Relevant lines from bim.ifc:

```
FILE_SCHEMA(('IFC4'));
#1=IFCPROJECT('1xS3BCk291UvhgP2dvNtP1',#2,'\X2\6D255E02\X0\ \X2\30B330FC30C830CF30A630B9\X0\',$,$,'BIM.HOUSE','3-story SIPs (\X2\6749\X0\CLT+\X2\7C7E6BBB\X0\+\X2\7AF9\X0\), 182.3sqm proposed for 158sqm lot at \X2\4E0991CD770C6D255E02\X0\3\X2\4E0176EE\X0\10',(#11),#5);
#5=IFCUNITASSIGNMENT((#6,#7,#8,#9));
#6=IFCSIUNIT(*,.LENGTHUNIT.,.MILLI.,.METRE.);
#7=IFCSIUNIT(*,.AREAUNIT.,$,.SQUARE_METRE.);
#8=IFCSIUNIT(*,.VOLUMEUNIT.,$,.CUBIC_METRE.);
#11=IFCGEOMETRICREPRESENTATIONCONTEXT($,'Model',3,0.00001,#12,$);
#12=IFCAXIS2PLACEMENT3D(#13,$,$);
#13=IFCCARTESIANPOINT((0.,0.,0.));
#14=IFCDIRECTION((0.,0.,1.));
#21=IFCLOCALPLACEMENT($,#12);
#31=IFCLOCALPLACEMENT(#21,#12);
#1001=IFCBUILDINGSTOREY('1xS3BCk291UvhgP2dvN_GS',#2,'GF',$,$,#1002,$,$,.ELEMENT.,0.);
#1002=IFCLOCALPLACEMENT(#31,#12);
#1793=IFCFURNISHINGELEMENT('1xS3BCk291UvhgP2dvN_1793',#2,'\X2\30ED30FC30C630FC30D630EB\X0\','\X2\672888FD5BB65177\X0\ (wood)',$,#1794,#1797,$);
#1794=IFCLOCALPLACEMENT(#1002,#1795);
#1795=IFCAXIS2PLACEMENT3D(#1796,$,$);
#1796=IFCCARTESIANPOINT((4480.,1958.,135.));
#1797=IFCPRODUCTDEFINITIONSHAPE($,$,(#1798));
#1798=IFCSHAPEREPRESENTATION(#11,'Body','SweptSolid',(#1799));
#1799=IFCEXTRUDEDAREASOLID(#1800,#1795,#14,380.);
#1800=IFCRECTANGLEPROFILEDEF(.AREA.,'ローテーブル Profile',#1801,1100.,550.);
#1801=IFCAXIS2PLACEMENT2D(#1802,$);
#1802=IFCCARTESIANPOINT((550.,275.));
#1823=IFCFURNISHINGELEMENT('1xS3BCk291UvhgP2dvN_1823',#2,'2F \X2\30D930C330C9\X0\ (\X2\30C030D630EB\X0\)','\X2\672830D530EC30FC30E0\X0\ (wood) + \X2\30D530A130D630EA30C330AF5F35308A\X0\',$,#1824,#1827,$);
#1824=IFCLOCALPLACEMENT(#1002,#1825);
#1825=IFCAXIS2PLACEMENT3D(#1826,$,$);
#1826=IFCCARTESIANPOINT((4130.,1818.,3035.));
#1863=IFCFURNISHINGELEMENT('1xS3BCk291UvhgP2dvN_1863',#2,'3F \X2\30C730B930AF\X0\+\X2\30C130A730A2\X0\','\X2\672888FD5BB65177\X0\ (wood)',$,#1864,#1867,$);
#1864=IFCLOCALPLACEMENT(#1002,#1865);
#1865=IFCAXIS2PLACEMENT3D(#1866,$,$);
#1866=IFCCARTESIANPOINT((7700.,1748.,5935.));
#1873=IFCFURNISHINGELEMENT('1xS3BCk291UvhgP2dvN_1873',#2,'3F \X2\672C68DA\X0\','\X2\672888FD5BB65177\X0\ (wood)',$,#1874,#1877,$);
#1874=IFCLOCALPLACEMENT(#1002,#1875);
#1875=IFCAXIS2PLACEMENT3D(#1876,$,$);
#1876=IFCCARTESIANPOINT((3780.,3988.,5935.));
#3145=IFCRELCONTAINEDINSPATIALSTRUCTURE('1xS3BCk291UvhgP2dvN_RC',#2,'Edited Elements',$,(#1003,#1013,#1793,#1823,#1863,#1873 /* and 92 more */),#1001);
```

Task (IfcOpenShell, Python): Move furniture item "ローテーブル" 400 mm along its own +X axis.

```python
import ifcopenshell
import ifcopenshell.api.geometry
import ifcopenshell.util.placement
import ifcopenshell.util.unit

model = ifcopenshell.open("bim.ifc")
unit_scale = ifcopenshell.util.unit.calculate_unit_scale(model)

item = model.by_id(1793)
matrix = ifcopenshell.util.placement.get_local_placement(item.ObjectPlacement)
matrix[:3, 3] += matrix[:3, 0] * 0.4 / unit_scale
ifcopenshell.api.geometry.edit_object_placement(model, product=item, matrix=matrix, is_si=False)

print(ifcopenshell.util.placement.get_local_placement(item.ObjectPlacement).round(3) + 0.0)

model.write("bim_v2.ifc")
```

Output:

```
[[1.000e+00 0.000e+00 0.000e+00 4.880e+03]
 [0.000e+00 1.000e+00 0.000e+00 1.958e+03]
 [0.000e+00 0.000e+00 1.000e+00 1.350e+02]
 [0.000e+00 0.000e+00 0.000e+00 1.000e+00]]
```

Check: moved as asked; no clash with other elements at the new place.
